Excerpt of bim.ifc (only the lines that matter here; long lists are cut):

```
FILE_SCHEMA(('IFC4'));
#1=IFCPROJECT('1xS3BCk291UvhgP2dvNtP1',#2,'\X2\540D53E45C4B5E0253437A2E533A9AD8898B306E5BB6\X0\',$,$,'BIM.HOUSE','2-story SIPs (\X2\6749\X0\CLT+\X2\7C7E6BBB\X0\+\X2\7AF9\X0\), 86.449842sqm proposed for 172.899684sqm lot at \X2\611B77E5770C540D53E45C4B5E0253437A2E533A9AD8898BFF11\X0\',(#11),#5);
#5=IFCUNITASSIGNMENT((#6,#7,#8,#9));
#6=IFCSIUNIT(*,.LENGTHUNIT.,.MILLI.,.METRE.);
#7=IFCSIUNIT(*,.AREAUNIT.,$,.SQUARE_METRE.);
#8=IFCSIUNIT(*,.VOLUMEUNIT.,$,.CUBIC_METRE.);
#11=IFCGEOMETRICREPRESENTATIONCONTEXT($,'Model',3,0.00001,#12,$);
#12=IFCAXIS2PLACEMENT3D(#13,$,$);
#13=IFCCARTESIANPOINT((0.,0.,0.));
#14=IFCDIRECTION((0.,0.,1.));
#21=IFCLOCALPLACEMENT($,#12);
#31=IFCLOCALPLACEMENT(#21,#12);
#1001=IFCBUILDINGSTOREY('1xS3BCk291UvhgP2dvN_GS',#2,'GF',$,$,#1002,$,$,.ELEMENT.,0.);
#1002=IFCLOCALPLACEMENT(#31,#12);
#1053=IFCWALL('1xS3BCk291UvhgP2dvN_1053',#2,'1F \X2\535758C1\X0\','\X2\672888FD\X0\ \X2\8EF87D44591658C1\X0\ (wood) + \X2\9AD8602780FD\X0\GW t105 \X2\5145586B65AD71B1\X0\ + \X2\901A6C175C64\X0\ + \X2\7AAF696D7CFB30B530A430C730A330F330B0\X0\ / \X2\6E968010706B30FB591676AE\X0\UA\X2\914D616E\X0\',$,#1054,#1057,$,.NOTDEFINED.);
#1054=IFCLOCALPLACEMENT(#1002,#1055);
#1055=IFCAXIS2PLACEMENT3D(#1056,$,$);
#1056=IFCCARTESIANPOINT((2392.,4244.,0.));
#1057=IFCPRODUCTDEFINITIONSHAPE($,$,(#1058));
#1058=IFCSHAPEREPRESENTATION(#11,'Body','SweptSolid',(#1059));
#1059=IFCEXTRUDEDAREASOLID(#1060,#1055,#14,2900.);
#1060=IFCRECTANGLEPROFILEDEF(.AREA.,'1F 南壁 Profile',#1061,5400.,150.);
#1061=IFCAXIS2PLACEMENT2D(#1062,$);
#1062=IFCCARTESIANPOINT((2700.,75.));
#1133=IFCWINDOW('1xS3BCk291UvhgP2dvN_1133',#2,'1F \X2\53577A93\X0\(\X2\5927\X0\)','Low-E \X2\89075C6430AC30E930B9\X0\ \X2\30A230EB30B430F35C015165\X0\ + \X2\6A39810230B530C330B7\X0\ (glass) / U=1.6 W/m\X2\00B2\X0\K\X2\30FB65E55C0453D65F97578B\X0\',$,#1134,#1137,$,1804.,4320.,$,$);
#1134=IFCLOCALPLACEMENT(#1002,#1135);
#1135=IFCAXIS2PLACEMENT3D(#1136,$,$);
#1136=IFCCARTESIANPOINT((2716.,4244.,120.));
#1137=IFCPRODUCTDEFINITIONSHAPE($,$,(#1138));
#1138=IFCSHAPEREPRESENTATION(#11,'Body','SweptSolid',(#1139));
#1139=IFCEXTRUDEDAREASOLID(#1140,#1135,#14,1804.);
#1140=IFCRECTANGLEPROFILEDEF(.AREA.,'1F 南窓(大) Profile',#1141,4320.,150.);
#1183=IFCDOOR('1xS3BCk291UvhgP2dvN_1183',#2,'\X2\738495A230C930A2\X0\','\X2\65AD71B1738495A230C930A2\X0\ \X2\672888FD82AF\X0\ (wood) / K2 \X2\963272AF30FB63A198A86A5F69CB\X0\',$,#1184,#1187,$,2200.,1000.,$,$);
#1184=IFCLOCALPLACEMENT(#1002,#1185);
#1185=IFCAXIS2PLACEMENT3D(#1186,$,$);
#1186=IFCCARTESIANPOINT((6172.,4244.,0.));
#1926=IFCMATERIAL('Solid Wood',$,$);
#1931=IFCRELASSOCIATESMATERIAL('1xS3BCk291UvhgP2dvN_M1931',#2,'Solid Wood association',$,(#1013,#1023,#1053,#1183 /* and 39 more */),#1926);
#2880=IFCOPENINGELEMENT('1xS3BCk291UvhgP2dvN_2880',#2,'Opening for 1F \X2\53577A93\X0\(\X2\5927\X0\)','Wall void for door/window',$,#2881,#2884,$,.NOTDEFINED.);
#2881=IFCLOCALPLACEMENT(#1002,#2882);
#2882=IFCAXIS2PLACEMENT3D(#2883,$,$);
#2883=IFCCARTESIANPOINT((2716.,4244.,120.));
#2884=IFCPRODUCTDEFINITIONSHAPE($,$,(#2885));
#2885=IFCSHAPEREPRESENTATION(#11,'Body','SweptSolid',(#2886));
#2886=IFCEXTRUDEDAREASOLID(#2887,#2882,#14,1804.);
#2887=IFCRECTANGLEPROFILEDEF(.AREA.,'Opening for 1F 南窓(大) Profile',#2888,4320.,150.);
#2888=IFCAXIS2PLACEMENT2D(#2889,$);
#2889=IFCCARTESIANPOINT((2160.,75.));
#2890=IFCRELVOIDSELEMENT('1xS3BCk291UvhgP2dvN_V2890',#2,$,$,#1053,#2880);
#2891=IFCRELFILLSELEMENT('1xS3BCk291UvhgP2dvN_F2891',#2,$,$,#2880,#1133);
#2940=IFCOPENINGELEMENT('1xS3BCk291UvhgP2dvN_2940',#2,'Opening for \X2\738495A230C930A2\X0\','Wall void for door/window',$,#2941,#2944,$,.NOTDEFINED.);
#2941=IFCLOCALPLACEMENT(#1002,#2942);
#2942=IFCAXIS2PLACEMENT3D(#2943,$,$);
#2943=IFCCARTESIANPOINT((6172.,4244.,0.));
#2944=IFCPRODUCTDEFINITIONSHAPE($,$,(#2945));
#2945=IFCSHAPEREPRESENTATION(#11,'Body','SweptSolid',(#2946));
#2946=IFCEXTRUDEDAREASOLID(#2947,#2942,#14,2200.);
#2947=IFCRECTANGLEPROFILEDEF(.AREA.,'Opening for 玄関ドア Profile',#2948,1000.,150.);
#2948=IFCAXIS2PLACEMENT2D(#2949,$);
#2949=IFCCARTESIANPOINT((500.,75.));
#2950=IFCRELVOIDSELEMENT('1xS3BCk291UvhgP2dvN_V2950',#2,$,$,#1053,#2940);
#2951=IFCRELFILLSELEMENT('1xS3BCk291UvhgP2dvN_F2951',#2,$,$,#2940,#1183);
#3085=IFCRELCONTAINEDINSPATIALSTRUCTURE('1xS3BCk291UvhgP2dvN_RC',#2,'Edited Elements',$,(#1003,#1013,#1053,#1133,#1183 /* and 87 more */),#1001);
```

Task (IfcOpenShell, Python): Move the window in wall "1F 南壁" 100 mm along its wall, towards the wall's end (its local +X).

```python
import ifcopenshell
import ifcopenshell.api.geometry
import ifcopenshell.util.placement
import ifcopenshell.util.unit

model = ifcopenshell.open("bim.ifc")
unit_scale = ifcopenshell.util.unit.calculate_unit_scale(model)

window = model.by_guid("1xS3BCk291UvhgP2dvN_1133")
opening = window.FillsVoids[0].RelatingOpeningElement
wall = opening.VoidsElements[0].RelatingBuildingElement

wall_matrix = ifcopenshell.util.placement.get_local_placement(wall.ObjectPlacement)
shift = wall_matrix[:3, 0] * 0.1 / unit_scale
before = ifcopenshell.util.placement.get_local_placement(window.ObjectPlacement)[:3, 3].copy()

# The window is not placed relative to its opening, so move both.
for product in (opening, window):
    matrix = ifcopenshell.util.placement.get_local_placement(product.ObjectPlacement)
    matrix[:3, 3] += shift
    ifcopenshell.api.geometry.edit_object_placement(model, product=product, matrix=matrix, is_si=False)

after = ifcopenshell.util.placement.get_local_placement(window.ObjectPlacement)[:3, 3]
print("window moved by", (after - before).round(3) + 0.0)

model.write("bim_updated.ifc")
```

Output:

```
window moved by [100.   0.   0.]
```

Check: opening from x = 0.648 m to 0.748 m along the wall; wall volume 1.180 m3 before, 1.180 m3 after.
